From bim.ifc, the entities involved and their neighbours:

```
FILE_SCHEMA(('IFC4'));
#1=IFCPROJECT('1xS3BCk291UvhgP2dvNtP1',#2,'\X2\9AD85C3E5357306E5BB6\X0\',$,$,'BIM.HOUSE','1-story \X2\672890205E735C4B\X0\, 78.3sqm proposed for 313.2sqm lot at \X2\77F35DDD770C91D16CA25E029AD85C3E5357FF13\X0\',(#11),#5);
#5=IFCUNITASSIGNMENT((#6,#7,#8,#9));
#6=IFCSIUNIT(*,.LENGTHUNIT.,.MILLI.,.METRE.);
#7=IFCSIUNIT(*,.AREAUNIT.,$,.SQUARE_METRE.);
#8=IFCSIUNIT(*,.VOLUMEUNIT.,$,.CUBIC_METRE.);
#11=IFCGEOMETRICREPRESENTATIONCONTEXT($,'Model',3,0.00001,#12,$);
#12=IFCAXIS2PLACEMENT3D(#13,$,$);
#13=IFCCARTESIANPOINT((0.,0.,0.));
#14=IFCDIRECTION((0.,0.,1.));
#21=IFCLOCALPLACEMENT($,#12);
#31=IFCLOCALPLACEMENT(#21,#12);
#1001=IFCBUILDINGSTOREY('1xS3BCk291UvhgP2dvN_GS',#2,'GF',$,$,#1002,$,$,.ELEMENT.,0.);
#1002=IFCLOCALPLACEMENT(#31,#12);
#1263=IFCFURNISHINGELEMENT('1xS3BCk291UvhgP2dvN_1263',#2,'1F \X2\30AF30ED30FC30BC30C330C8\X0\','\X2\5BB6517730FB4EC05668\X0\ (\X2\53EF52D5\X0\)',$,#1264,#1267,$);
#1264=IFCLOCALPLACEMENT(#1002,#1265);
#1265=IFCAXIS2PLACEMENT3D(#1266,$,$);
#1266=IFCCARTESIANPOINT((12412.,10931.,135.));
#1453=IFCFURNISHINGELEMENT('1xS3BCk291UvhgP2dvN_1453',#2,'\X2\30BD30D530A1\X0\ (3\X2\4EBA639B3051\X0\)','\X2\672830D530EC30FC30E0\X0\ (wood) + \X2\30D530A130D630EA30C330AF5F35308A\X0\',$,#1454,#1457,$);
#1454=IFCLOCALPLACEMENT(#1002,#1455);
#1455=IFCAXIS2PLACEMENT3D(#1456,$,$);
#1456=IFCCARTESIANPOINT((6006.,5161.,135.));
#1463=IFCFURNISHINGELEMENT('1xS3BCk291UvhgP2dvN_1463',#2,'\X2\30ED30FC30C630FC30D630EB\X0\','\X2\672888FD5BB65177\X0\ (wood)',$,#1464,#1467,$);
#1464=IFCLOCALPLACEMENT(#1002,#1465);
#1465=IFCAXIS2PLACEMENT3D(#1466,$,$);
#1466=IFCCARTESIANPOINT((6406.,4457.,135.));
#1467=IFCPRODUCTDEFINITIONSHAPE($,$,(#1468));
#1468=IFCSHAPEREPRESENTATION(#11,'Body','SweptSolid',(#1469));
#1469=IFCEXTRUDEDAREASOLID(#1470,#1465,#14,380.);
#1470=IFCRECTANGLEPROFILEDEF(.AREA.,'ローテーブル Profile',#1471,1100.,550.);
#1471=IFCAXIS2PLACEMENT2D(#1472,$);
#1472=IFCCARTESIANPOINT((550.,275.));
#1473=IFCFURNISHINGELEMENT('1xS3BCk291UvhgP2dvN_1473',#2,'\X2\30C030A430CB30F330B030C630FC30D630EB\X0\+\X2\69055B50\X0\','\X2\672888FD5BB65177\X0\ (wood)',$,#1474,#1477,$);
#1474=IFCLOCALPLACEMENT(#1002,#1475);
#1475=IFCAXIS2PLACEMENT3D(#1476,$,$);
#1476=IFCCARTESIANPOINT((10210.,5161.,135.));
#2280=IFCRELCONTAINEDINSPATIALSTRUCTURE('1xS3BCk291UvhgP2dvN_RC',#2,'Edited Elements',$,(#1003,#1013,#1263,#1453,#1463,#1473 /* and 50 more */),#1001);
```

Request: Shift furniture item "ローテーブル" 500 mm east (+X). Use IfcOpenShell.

```python
import ifcopenshell
import ifcopenshell.api.geometry
import ifcopenshell.util.placement
import ifcopenshell.util.unit

model = ifcopenshell.open("bim.ifc")
unit_scale = ifcopenshell.util.unit.calculate_unit_scale(model)

item = model.by_id(1463)
matrix = ifcopenshell.util.placement.get_local_placement(item.ObjectPlacement)
matrix[0, 3] += 0.5 / unit_scale
ifcopenshell.api.geometry.edit_object_placement(model, product=item, matrix=matrix, is_si=False)

print(ifcopenshell.util.placement.get_local_placement(item.ObjectPlacement).round(3) + 0.0)

model.write("bim-out.ifc")
```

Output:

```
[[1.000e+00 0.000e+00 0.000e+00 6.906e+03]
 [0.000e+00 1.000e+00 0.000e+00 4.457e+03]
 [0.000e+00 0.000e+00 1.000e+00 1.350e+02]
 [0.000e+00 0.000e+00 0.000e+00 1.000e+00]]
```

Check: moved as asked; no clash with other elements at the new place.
